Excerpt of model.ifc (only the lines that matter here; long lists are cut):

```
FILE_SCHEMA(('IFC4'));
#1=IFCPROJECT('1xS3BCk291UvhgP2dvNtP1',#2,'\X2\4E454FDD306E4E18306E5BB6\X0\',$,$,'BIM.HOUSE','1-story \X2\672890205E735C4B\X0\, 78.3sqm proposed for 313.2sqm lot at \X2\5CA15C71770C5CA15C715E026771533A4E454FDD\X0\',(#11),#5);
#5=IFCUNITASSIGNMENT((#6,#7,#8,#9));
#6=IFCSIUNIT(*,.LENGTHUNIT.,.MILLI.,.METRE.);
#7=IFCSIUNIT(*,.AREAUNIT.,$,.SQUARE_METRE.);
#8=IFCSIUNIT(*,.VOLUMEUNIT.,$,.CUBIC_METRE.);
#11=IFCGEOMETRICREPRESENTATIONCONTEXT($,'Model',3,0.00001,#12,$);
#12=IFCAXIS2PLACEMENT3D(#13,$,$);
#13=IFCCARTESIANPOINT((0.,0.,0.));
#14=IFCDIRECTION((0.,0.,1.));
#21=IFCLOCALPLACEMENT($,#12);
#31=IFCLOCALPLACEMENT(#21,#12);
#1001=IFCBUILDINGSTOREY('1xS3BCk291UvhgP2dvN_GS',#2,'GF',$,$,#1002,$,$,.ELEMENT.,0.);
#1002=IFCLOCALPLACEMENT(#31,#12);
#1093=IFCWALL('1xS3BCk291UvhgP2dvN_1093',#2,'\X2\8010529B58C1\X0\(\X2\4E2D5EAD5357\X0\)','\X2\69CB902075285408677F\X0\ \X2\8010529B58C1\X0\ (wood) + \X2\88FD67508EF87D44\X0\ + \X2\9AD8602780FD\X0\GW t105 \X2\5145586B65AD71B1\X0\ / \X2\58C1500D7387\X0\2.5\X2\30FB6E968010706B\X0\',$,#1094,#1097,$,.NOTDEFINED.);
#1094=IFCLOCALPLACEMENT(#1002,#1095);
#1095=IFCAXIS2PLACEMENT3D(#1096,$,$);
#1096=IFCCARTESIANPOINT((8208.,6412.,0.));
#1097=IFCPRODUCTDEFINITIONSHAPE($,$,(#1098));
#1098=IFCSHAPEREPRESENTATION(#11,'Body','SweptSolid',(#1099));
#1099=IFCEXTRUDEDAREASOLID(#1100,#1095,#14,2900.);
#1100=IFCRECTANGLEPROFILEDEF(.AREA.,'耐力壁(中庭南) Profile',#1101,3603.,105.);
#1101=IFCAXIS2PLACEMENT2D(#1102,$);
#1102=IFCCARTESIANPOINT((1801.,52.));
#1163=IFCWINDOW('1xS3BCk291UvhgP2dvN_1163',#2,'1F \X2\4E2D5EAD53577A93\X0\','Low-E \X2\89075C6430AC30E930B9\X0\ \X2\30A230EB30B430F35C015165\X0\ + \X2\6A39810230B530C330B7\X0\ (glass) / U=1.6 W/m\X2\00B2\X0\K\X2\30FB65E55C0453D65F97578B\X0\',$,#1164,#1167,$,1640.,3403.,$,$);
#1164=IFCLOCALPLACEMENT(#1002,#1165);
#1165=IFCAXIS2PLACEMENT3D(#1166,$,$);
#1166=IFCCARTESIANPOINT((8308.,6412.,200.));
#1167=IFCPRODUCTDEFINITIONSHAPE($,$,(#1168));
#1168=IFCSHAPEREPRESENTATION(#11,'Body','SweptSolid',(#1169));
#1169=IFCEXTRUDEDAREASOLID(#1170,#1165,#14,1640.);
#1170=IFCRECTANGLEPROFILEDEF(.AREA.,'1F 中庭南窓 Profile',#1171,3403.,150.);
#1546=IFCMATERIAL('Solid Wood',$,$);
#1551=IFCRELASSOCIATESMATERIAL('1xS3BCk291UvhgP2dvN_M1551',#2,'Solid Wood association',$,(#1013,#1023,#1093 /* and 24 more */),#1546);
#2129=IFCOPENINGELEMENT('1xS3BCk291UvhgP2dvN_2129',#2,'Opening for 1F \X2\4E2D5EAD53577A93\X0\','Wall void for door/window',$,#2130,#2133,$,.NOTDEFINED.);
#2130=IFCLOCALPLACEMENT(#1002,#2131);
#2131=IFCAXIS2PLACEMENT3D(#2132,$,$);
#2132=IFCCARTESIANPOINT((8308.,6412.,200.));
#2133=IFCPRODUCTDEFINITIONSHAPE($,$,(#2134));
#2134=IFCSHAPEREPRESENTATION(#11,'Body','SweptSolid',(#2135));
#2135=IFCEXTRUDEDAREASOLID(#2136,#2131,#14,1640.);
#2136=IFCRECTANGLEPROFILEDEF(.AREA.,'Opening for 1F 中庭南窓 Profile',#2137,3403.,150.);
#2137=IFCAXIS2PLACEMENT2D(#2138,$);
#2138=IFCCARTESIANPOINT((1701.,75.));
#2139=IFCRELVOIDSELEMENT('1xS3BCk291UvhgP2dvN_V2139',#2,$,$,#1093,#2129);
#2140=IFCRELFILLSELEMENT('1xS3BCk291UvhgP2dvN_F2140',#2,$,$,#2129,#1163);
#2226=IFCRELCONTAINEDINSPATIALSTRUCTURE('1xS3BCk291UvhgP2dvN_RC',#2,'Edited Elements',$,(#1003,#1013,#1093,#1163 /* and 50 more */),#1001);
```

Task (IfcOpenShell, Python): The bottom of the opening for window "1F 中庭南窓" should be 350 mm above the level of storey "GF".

```python
import numpy as np
import ifcopenshell
import ifcopenshell.api.geometry
import ifcopenshell.geom
import ifcopenshell.util.element
import ifcopenshell.util.placement
import ifcopenshell.util.shape
import ifcopenshell.util.unit

model = ifcopenshell.open("model.ifc")
unit_scale = ifcopenshell.util.unit.calculate_unit_scale(model)

window = model.by_guid("1xS3BCk291UvhgP2dvN_1163")
opening = window.FillsVoids[0].RelatingOpeningElement
storey = ifcopenshell.util.element.get_container(window, ifc_class="IfcBuildingStorey")
level = ifcopenshell.util.placement.get_local_placement(storey.ObjectPlacement)[2, 3]

# The opening's origin need not be at the sill, so measure its lowest point.
shape = ifcopenshell.geom.create_shape(ifcopenshell.geom.settings(), opening)
bottom = ifcopenshell.util.shape.get_shape_bottom_elevation(shape, shape.geometry) / unit_scale
dz = level + 0.35 / unit_scale - bottom

shift = np.array([0.0, 0.0, dz])
# The window is not placed relative to its opening, so move both.
for product in (opening, window):
    matrix = ifcopenshell.util.placement.get_local_placement(product.ObjectPlacement)
    matrix[:3, 3] += shift
    ifcopenshell.api.geometry.edit_object_placement(model, product=product, matrix=matrix, is_si=False)

print(f"moved by {dz * unit_scale:+.3f} m")

model.write("model_rev.ifc")
```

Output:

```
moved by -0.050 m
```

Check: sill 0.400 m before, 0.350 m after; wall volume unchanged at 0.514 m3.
